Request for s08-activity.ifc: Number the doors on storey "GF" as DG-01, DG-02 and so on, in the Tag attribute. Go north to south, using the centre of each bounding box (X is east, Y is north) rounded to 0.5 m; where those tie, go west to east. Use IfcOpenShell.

First a look at what the model holds.

```python
import ifcopenshell
import ifcopenshell.util.element
import ifcopenshell.util.placement

model = ifcopenshell.open("s08-activity.ifc")
print(model.schema)
storey = next(s for s in model.by_type("IfcBuildingStorey") if s.Name == "GF")
doors = [e for e in ifcopenshell.util.element.get_decomposition(storey) if e.is_a("IfcDoor")]
for e in sorted(doors, key=lambda e: e.id()):
    origin = ifcopenshell.util.placement.get_local_placement(e.ObjectPlacement)[:3, 3]
    print(e.id(), e.Tag, e.Name, origin.round(2) + 0.0, sep=" | ")
```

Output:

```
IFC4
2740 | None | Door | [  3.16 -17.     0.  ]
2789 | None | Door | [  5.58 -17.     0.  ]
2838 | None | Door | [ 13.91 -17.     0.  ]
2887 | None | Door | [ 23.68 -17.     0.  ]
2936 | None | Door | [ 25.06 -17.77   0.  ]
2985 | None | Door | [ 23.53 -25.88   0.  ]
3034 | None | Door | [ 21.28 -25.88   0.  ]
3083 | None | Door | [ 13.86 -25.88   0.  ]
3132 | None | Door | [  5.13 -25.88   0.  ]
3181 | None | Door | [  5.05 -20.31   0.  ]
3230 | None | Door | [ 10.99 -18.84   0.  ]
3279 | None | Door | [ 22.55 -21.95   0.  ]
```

```python
import ifcopenshell
import ifcopenshell.geom
import ifcopenshell.util.element
import ifcopenshell.util.shape

model = ifcopenshell.open("s08-activity.ifc")
settings = ifcopenshell.geom.settings()
settings.set("use-world-coords", True)


def centre(element):
    shape = ifcopenshell.geom.create_shape(settings, element)
    return ifcopenshell.util.shape.get_bbox_centroid(shape.geometry)


storey = next(s for s in model.by_type("IfcBuildingStorey") if s.Name == "GF")
doors = [e for e in ifcopenshell.util.element.get_decomposition(storey) if e.is_a("IfcDoor")]

# Insertion points can sit at a corner or the storey origin, so sort by the geometry (in metres).
centres = {e: centre(e) for e in doors}
doors.sort(key=lambda e: (-round(centres[e][1] / 0.5), centres[e][0]))

for i, e in enumerate(doors, start=1):
    number = f"DG-{i:02d}"
    e.Tag = number
    print(e.id(), number)

model.write("s08-activity_v2.ifc")
```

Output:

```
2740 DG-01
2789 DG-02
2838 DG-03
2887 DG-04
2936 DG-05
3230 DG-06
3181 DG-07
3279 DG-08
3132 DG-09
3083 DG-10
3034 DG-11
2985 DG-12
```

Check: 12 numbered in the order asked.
